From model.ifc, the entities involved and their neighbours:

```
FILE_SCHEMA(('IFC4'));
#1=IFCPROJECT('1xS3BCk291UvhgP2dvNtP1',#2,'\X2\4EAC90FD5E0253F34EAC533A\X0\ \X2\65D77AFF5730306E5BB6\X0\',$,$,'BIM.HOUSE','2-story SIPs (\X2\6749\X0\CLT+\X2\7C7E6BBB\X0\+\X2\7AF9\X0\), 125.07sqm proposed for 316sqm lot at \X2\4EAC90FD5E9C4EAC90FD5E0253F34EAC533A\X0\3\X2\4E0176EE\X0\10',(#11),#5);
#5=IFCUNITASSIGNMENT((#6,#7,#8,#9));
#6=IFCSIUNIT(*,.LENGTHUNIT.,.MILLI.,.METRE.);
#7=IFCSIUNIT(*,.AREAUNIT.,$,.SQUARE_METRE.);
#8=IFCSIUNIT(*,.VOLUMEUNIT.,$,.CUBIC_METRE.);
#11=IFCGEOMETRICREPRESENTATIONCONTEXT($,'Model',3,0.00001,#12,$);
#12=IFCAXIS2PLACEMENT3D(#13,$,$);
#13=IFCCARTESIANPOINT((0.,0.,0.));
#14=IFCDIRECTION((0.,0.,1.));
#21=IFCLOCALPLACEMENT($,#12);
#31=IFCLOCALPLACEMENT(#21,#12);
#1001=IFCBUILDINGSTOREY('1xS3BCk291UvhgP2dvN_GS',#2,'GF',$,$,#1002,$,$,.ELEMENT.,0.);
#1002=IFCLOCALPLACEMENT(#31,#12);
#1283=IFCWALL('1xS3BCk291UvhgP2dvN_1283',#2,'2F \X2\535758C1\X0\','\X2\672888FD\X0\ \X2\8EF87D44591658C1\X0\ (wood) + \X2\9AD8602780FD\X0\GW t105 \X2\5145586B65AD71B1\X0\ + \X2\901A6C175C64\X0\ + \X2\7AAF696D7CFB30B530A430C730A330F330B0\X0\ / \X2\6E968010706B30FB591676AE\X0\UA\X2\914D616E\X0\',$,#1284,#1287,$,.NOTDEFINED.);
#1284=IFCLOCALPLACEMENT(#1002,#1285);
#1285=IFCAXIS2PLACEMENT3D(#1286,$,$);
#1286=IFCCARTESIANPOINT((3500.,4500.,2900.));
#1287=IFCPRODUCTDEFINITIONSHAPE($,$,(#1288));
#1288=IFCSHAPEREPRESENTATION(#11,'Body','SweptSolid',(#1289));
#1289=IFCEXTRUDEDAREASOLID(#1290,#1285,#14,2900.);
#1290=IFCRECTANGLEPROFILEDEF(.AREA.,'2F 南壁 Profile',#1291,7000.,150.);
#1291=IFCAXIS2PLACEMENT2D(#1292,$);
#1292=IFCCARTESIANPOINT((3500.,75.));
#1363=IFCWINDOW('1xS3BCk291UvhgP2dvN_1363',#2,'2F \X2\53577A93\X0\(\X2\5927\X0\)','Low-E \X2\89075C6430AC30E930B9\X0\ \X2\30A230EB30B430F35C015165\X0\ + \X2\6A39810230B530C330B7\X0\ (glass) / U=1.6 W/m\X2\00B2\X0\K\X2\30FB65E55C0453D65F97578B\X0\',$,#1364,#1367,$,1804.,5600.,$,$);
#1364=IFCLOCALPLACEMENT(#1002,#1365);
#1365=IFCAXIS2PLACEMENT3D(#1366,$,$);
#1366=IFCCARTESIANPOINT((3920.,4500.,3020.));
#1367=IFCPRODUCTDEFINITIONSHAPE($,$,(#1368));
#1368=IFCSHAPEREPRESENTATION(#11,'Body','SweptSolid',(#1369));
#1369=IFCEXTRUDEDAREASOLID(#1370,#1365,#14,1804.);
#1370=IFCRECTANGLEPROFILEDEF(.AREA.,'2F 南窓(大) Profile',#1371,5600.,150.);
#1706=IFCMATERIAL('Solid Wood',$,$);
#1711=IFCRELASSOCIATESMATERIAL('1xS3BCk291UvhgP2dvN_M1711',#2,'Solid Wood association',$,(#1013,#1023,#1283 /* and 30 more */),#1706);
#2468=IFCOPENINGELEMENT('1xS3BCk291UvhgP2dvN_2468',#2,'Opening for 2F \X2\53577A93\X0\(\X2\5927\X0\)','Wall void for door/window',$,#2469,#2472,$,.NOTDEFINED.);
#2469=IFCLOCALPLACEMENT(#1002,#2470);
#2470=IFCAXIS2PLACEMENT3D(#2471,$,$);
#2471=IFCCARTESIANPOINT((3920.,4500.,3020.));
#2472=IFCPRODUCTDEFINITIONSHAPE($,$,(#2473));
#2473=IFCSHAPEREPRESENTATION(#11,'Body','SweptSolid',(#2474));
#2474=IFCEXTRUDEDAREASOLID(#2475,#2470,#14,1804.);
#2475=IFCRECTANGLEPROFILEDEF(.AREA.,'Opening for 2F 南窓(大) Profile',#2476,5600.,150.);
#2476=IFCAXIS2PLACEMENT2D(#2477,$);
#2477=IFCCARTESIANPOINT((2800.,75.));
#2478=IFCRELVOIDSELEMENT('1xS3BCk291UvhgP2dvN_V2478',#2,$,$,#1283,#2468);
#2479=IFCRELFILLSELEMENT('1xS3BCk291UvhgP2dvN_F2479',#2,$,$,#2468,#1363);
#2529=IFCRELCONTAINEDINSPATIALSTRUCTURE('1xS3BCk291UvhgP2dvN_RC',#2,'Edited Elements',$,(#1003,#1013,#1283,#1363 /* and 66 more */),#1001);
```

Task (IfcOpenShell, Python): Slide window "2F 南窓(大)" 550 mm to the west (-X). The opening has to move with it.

```python
import ifcopenshell
import ifcopenshell.api.geometry
import ifcopenshell.util.placement
import ifcopenshell.util.unit

model = ifcopenshell.open("model.ifc")
unit_scale = ifcopenshell.util.unit.calculate_unit_scale(model)

window = model.by_guid("1xS3BCk291UvhgP2dvN_1363")
opening = window.FillsVoids[0].RelatingOpeningElement
wall = opening.VoidsElements[0].RelatingBuildingElement

wall_matrix = ifcopenshell.util.placement.get_local_placement(wall.ObjectPlacement)
shift = wall_matrix[:3, 0] * -0.55 / unit_scale
before = ifcopenshell.util.placement.get_local_placement(window.ObjectPlacement)[:3, 3].copy()

# The window is not placed relative to its opening, so move both.
for product in (opening, window):
    matrix = ifcopenshell.util.placement.get_local_placement(product.ObjectPlacement)
    matrix[:3, 3] += shift
    ifcopenshell.api.geometry.edit_object_placement(model, product=product, matrix=matrix, is_si=False)

after = ifcopenshell.util.placement.get_local_placement(window.ObjectPlacement)[:3, 3]
print("window moved by", (after - before).round(3) + 0.0)

model.write("model_v2.ifc")
```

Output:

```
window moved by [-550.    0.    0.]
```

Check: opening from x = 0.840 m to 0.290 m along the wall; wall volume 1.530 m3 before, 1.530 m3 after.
